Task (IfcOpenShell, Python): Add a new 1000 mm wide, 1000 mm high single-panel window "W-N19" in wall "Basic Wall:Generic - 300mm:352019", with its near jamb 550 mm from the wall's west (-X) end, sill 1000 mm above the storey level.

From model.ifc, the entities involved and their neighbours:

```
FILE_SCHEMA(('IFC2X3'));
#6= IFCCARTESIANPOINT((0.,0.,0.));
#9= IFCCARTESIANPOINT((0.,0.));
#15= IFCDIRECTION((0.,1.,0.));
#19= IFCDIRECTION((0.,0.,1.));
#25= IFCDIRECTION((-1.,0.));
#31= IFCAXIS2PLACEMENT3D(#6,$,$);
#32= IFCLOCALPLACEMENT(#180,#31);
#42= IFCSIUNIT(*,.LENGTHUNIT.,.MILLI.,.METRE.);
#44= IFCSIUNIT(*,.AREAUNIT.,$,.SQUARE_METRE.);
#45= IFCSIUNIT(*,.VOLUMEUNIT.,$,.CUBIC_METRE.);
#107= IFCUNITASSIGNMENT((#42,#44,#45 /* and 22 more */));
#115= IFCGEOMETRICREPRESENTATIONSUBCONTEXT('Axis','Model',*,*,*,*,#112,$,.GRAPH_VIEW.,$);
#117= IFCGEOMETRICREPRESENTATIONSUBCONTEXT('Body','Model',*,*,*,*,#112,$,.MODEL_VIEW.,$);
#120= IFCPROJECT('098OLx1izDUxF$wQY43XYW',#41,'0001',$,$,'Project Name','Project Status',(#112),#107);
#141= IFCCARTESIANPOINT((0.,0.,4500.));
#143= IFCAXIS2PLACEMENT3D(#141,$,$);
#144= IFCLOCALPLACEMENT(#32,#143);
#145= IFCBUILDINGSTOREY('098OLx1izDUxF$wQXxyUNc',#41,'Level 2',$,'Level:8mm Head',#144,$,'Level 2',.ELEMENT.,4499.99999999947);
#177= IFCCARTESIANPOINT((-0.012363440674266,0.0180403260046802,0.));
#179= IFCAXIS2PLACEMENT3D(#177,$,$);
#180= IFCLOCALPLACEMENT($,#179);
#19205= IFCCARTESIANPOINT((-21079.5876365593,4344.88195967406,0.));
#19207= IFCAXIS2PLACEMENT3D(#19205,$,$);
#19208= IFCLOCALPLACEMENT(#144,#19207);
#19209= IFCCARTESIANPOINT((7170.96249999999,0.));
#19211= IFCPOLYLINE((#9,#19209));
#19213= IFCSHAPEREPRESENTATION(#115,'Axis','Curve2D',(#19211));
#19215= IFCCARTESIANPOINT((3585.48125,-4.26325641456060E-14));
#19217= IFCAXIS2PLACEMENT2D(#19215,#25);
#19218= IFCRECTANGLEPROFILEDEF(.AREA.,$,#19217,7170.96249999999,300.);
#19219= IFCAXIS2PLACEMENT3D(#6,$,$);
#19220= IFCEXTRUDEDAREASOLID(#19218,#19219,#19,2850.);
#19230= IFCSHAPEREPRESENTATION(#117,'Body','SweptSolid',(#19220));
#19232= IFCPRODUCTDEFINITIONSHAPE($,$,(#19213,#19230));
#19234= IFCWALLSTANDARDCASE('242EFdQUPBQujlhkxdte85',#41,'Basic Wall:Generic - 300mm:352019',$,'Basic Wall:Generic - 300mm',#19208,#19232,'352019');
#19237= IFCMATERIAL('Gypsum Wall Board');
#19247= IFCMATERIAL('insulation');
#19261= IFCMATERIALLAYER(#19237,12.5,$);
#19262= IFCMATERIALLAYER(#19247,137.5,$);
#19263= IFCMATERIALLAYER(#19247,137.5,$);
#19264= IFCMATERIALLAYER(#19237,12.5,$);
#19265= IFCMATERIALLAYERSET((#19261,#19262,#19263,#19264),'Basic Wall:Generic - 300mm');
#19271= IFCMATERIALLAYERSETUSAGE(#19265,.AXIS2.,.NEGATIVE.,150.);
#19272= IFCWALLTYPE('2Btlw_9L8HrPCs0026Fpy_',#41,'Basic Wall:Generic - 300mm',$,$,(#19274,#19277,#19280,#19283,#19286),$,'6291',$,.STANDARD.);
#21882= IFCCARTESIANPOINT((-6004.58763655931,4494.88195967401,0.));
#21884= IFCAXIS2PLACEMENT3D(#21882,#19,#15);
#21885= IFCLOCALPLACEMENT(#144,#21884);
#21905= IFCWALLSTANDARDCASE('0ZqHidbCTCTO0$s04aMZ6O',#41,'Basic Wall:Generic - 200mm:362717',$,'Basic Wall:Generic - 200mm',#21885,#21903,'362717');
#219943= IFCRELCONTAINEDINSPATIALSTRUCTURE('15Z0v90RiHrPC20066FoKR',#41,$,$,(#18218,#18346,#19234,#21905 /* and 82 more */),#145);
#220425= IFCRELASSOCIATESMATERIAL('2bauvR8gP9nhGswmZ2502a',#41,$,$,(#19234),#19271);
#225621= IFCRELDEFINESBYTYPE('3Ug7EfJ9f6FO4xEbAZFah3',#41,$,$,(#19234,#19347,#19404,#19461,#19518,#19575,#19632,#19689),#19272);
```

```python
import numpy as np
import ifcopenshell
import ifcopenshell.api.feature
import ifcopenshell.api.geometry
import ifcopenshell.api.root
import ifcopenshell.api.spatial
import ifcopenshell.api.type
import ifcopenshell.geom
import ifcopenshell.util.element
import ifcopenshell.util.placement
import ifcopenshell.util.representation
import ifcopenshell.util.shape
import ifcopenshell.util.unit

model = ifcopenshell.open("model.ifc")
unit_scale = ifcopenshell.util.unit.calculate_unit_scale(model)
settings = ifcopenshell.geom.settings()


def volume(element):
    """Net volume in cubic metres, openings subtracted."""
    shape = ifcopenshell.geom.create_shape(settings, element)
    return ifcopenshell.util.shape.get_volume(shape.geometry)


wall = model.by_guid("242EFdQUPBQujlhkxdte85")
storey = ifcopenshell.util.element.get_container(wall, ifc_class="IfcBuildingStorey")
context = ifcopenshell.util.representation.get_context(model, "Model", "Body", "MODEL_VIEW")
before = volume(wall)

width, height, from_end, sill = 1, 1, 0.55, 1  # metres

# The wall runs along its own X axis, and the end named is its -X end.
wall_shape = ifcopenshell.geom.create_shape(settings, wall)
x, y, z = ifcopenshell.util.shape.get_vertices(wall_shape.geometry).T
start = x.min() + from_end
face, thickness = float(y.min()), float(y.max() - y.min())
wall_matrix = ifcopenshell.util.placement.get_local_placement(wall.ObjectPlacement)
level = ifcopenshell.util.placement.get_local_placement(storey.ObjectPlacement)[2, 3]


def in_wall(x, y):
    """Placement at x, y metres in the wall's axes, at sill height."""
    matrix = wall_matrix.copy()
    matrix[:, 3] = wall_matrix @ np.array([x / unit_scale, y / unit_scale, 0.0, 1.0])
    matrix[2, 3] = level + sill / unit_scale
    return matrix


# Opening: a box that overshoots both wall faces by 50 mm.
opening = ifcopenshell.api.root.create_entity(model, ifc_class="IfcOpeningElement")
box = ifcopenshell.api.geometry.add_wall_representation(
    model, context=context, length=width, height=height, thickness=thickness + 0.1
)
ifcopenshell.api.geometry.assign_representation(model, product=opening, representation=box)
ifcopenshell.api.geometry.edit_object_placement(model, product=opening, matrix=in_wall(start, face - 0.05), is_si=False)
ifcopenshell.api.feature.add_feature(model, feature=opening, element=wall)

window = ifcopenshell.api.root.create_entity(model, ifc_class="IfcWindow", name="W-N19")
window.OverallWidth, window.OverallHeight = width / unit_scale, height / unit_scale
body = ifcopenshell.api.geometry.add_window_representation(
    model,
    context=context,
    overall_width=window.OverallWidth,
    overall_height=window.OverallHeight,
    partition_type="SINGLE_PANEL",
)
ifcopenshell.api.geometry.assign_representation(model, product=window, representation=body)
ifcopenshell.api.spatial.assign_container(model, products=[window], relating_structure=storey)
fills = ifcopenshell.api.feature.add_filling(model, opening=opening, element=window)
fills.OwnerHistory = window.OwnerHistory  # required in IFC2X3

# IFC2X3 keeps the operation on the window style.
style = ifcopenshell.api.root.create_entity(model, ifc_class="IfcWindowStyle", name="W-N19")
style.OperationType, style.ConstructionType = "SINGLE_PANEL", "NOTDEFINED"
style.ParameterTakesPrecedence = style.Sizeable = False
ifcopenshell.api.type.assign_type(model, related_objects=[window], relating_type=style)

# Centre the window in the wall's thickness.
ifcopenshell.api.geometry.edit_object_placement(model, product=window, matrix=in_wall(start, face), is_si=False)
window_shape = ifcopenshell.geom.create_shape(settings, window)
depth = ifcopenshell.util.shape.get_vertices(window_shape.geometry)[:, 1]
offset = face + thickness / 2 - (depth.min() + depth.max()) / 2
ifcopenshell.api.geometry.edit_object_placement(model, product=window, matrix=in_wall(start, offset), is_si=False)

after = volume(wall)

print(f"wall volume {before:.3f} -> {after:.3f} m3")

model.write("model_rev.ifc")
```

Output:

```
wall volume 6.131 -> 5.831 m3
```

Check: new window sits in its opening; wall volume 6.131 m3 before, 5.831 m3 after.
